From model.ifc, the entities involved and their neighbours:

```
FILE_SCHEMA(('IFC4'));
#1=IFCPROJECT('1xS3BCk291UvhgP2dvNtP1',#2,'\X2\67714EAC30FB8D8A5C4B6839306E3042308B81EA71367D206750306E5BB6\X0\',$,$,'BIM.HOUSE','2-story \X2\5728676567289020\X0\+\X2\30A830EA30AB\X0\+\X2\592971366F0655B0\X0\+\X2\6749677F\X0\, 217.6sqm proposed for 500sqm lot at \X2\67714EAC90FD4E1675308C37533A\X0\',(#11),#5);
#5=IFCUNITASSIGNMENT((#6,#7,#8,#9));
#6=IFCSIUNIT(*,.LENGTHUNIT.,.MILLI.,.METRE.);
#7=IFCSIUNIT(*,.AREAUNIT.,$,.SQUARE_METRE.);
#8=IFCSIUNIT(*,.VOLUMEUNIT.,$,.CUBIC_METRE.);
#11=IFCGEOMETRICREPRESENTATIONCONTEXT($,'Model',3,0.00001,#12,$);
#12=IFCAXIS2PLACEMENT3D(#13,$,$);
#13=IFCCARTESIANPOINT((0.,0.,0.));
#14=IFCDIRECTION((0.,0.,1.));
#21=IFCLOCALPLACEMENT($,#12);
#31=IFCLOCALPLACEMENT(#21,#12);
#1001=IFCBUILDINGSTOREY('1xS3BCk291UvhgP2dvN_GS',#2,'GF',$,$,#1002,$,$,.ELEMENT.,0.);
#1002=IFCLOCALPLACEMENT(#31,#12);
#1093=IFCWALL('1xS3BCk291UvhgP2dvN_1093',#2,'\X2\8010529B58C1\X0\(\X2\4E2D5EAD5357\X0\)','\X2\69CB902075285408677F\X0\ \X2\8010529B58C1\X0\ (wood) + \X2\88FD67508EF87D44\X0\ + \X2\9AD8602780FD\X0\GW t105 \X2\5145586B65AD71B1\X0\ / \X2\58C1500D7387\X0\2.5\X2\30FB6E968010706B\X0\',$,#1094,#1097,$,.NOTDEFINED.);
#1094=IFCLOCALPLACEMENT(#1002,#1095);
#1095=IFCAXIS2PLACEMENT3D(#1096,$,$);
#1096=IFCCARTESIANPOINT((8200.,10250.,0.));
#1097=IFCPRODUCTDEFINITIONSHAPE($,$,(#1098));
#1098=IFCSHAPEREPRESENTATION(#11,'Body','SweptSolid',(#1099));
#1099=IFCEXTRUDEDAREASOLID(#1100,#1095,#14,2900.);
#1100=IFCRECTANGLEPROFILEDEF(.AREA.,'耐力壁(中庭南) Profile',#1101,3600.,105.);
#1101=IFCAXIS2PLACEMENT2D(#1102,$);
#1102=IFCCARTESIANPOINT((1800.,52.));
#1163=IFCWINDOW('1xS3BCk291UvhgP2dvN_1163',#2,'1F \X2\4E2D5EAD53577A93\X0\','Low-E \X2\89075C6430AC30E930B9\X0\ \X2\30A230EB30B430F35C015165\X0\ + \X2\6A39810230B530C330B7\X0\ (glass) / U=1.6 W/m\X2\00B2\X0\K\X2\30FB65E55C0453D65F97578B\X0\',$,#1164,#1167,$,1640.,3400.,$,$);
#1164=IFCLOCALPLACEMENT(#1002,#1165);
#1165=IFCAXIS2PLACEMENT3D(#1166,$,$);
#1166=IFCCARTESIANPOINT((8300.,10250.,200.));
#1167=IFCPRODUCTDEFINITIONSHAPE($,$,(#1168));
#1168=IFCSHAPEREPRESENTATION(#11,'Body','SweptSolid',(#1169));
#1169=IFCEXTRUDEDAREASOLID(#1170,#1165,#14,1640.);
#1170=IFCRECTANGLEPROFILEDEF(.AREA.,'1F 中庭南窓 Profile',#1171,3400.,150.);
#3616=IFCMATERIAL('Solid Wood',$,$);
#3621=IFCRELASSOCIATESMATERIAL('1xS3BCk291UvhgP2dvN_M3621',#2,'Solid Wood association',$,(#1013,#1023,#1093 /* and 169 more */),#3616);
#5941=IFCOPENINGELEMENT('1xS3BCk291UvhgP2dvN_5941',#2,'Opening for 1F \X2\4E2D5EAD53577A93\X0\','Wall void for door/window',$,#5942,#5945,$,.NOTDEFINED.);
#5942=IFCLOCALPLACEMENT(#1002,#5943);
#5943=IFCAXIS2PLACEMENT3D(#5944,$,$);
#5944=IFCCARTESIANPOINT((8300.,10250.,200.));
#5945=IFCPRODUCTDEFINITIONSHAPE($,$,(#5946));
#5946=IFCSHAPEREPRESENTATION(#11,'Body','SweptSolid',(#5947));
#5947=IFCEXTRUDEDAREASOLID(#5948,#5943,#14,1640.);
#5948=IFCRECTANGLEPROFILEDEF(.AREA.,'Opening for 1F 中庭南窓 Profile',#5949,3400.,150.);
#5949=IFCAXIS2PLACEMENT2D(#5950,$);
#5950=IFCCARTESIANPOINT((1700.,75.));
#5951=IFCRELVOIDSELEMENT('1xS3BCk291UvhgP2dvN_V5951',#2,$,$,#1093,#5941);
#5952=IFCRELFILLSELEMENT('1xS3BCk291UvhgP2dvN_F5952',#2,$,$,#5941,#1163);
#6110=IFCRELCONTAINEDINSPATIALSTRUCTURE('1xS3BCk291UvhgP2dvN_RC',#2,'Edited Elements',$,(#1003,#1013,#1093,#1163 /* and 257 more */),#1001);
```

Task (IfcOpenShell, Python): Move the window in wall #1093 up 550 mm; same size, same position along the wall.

```python
import numpy as np
import ifcopenshell
import ifcopenshell.api.geometry
import ifcopenshell.util.placement
import ifcopenshell.util.unit

model = ifcopenshell.open("model.ifc")
unit_scale = ifcopenshell.util.unit.calculate_unit_scale(model)

window = model.by_id(1163)
opening = window.FillsVoids[0].RelatingOpeningElement
dz = 0.55 / unit_scale

shift = np.array([0.0, 0.0, dz])
# The window is not placed relative to its opening, so move both.
for product in (opening, window):
    matrix = ifcopenshell.util.placement.get_local_placement(product.ObjectPlacement)
    matrix[:3, 3] += shift
    ifcopenshell.api.geometry.edit_object_placement(model, product=product, matrix=matrix, is_si=False)

print(f"moved by {dz * unit_scale:+.3f} m")

model.write("model-out.ifc")
```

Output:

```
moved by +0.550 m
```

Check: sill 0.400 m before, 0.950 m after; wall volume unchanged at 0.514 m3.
